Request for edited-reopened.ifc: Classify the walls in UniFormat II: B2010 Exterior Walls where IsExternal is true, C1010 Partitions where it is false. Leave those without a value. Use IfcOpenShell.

First a look at what the model holds.

```python
import ifcopenshell
import ifcopenshell.util.element

model = ifcopenshell.open("edited-reopened.ifc")
print(model.schema)
print("classifications:", [c.Name for c in model.by_type("IfcClassification")])
values = [ifcopenshell.util.element.get_pset(e, "Pset_WallCommon", "IsExternal") for e in model.by_type("IfcWall")]
for value in (True, False, None):
    print("IsExternal", value, values.count(value))
```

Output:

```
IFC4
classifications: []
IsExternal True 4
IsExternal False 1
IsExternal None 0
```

```python
import ifcopenshell
import ifcopenshell.api.classification
import ifcopenshell.util.element

model = ifcopenshell.open("edited-reopened.ifc")

system = ifcopenshell.api.classification.add_classification(model, classification="UniFormat II")

walls = model.by_type("IfcWall")
external = {e: ifcopenshell.util.element.get_pset(e, "Pset_WallCommon", "IsExternal") for e in walls}
for flag, code, name in ((True, "B2010", "Exterior Walls"), (False, "C1010", "Partitions")):
    products = [e for e in walls if external[e] is flag]
    ifcopenshell.api.classification.add_reference(
        model, products=products, classification=system, identification=code, name=name
    )
    print(code, len(products))

model.write("edited-reopened_updated.ifc")
```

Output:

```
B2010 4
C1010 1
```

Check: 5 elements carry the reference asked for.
